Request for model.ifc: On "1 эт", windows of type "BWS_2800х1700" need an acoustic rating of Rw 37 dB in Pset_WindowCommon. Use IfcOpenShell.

First a look at what the model holds.

```python
import ifcopenshell
import ifcopenshell.util.element

model = ifcopenshell.open("model.ifc")
print(model.schema)
storey = next(s for s in model.by_type("IfcBuildingStorey") if s.Name == "1 эт")
windows = [e for e in ifcopenshell.util.element.get_decomposition(storey) if e.is_a("IfcWindow")]
seen = {}
for e in windows:
    element_type = ifcopenshell.util.element.get_type(e)
    key = (element_type.Name if element_type != e and element_type else None, ifcopenshell.util.element.get_pset(e, "Pset_WindowCommon", "AcousticRating"))
    seen[key] = seen.get(key, 0) + 1
for (name, value), count in sorted(seen.items(), key=str):
    print(count, "x", name, "|", value)
```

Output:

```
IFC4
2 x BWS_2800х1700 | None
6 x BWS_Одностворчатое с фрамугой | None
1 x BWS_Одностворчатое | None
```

```python
import ifcopenshell
import ifcopenshell.api.pset
import ifcopenshell.util.element

model = ifcopenshell.open("model.ifc")

storey = next(s for s in model.by_type("IfcBuildingStorey") if s.Name == "1 эт")
windows = [e for e in ifcopenshell.util.element.get_decomposition(storey) if e.is_a("IfcWindow")]

count = 0
for e in windows:
    element_type = ifcopenshell.util.element.get_type(e)
    if element_type in (None, e) or element_type.Name != "BWS_2800х1700":
        continue
    # add_pset returns the element's existing set when there is one.
    pset = ifcopenshell.api.pset.add_pset(model, product=e, name="Pset_WindowCommon")
    ifcopenshell.api.pset.edit_pset(model, pset=pset, properties={"AcousticRating": "Rw 37 dB"})
    count += 1

print(count, "windows updated")

model.write("model_edited.ifc")
```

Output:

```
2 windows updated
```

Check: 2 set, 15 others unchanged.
